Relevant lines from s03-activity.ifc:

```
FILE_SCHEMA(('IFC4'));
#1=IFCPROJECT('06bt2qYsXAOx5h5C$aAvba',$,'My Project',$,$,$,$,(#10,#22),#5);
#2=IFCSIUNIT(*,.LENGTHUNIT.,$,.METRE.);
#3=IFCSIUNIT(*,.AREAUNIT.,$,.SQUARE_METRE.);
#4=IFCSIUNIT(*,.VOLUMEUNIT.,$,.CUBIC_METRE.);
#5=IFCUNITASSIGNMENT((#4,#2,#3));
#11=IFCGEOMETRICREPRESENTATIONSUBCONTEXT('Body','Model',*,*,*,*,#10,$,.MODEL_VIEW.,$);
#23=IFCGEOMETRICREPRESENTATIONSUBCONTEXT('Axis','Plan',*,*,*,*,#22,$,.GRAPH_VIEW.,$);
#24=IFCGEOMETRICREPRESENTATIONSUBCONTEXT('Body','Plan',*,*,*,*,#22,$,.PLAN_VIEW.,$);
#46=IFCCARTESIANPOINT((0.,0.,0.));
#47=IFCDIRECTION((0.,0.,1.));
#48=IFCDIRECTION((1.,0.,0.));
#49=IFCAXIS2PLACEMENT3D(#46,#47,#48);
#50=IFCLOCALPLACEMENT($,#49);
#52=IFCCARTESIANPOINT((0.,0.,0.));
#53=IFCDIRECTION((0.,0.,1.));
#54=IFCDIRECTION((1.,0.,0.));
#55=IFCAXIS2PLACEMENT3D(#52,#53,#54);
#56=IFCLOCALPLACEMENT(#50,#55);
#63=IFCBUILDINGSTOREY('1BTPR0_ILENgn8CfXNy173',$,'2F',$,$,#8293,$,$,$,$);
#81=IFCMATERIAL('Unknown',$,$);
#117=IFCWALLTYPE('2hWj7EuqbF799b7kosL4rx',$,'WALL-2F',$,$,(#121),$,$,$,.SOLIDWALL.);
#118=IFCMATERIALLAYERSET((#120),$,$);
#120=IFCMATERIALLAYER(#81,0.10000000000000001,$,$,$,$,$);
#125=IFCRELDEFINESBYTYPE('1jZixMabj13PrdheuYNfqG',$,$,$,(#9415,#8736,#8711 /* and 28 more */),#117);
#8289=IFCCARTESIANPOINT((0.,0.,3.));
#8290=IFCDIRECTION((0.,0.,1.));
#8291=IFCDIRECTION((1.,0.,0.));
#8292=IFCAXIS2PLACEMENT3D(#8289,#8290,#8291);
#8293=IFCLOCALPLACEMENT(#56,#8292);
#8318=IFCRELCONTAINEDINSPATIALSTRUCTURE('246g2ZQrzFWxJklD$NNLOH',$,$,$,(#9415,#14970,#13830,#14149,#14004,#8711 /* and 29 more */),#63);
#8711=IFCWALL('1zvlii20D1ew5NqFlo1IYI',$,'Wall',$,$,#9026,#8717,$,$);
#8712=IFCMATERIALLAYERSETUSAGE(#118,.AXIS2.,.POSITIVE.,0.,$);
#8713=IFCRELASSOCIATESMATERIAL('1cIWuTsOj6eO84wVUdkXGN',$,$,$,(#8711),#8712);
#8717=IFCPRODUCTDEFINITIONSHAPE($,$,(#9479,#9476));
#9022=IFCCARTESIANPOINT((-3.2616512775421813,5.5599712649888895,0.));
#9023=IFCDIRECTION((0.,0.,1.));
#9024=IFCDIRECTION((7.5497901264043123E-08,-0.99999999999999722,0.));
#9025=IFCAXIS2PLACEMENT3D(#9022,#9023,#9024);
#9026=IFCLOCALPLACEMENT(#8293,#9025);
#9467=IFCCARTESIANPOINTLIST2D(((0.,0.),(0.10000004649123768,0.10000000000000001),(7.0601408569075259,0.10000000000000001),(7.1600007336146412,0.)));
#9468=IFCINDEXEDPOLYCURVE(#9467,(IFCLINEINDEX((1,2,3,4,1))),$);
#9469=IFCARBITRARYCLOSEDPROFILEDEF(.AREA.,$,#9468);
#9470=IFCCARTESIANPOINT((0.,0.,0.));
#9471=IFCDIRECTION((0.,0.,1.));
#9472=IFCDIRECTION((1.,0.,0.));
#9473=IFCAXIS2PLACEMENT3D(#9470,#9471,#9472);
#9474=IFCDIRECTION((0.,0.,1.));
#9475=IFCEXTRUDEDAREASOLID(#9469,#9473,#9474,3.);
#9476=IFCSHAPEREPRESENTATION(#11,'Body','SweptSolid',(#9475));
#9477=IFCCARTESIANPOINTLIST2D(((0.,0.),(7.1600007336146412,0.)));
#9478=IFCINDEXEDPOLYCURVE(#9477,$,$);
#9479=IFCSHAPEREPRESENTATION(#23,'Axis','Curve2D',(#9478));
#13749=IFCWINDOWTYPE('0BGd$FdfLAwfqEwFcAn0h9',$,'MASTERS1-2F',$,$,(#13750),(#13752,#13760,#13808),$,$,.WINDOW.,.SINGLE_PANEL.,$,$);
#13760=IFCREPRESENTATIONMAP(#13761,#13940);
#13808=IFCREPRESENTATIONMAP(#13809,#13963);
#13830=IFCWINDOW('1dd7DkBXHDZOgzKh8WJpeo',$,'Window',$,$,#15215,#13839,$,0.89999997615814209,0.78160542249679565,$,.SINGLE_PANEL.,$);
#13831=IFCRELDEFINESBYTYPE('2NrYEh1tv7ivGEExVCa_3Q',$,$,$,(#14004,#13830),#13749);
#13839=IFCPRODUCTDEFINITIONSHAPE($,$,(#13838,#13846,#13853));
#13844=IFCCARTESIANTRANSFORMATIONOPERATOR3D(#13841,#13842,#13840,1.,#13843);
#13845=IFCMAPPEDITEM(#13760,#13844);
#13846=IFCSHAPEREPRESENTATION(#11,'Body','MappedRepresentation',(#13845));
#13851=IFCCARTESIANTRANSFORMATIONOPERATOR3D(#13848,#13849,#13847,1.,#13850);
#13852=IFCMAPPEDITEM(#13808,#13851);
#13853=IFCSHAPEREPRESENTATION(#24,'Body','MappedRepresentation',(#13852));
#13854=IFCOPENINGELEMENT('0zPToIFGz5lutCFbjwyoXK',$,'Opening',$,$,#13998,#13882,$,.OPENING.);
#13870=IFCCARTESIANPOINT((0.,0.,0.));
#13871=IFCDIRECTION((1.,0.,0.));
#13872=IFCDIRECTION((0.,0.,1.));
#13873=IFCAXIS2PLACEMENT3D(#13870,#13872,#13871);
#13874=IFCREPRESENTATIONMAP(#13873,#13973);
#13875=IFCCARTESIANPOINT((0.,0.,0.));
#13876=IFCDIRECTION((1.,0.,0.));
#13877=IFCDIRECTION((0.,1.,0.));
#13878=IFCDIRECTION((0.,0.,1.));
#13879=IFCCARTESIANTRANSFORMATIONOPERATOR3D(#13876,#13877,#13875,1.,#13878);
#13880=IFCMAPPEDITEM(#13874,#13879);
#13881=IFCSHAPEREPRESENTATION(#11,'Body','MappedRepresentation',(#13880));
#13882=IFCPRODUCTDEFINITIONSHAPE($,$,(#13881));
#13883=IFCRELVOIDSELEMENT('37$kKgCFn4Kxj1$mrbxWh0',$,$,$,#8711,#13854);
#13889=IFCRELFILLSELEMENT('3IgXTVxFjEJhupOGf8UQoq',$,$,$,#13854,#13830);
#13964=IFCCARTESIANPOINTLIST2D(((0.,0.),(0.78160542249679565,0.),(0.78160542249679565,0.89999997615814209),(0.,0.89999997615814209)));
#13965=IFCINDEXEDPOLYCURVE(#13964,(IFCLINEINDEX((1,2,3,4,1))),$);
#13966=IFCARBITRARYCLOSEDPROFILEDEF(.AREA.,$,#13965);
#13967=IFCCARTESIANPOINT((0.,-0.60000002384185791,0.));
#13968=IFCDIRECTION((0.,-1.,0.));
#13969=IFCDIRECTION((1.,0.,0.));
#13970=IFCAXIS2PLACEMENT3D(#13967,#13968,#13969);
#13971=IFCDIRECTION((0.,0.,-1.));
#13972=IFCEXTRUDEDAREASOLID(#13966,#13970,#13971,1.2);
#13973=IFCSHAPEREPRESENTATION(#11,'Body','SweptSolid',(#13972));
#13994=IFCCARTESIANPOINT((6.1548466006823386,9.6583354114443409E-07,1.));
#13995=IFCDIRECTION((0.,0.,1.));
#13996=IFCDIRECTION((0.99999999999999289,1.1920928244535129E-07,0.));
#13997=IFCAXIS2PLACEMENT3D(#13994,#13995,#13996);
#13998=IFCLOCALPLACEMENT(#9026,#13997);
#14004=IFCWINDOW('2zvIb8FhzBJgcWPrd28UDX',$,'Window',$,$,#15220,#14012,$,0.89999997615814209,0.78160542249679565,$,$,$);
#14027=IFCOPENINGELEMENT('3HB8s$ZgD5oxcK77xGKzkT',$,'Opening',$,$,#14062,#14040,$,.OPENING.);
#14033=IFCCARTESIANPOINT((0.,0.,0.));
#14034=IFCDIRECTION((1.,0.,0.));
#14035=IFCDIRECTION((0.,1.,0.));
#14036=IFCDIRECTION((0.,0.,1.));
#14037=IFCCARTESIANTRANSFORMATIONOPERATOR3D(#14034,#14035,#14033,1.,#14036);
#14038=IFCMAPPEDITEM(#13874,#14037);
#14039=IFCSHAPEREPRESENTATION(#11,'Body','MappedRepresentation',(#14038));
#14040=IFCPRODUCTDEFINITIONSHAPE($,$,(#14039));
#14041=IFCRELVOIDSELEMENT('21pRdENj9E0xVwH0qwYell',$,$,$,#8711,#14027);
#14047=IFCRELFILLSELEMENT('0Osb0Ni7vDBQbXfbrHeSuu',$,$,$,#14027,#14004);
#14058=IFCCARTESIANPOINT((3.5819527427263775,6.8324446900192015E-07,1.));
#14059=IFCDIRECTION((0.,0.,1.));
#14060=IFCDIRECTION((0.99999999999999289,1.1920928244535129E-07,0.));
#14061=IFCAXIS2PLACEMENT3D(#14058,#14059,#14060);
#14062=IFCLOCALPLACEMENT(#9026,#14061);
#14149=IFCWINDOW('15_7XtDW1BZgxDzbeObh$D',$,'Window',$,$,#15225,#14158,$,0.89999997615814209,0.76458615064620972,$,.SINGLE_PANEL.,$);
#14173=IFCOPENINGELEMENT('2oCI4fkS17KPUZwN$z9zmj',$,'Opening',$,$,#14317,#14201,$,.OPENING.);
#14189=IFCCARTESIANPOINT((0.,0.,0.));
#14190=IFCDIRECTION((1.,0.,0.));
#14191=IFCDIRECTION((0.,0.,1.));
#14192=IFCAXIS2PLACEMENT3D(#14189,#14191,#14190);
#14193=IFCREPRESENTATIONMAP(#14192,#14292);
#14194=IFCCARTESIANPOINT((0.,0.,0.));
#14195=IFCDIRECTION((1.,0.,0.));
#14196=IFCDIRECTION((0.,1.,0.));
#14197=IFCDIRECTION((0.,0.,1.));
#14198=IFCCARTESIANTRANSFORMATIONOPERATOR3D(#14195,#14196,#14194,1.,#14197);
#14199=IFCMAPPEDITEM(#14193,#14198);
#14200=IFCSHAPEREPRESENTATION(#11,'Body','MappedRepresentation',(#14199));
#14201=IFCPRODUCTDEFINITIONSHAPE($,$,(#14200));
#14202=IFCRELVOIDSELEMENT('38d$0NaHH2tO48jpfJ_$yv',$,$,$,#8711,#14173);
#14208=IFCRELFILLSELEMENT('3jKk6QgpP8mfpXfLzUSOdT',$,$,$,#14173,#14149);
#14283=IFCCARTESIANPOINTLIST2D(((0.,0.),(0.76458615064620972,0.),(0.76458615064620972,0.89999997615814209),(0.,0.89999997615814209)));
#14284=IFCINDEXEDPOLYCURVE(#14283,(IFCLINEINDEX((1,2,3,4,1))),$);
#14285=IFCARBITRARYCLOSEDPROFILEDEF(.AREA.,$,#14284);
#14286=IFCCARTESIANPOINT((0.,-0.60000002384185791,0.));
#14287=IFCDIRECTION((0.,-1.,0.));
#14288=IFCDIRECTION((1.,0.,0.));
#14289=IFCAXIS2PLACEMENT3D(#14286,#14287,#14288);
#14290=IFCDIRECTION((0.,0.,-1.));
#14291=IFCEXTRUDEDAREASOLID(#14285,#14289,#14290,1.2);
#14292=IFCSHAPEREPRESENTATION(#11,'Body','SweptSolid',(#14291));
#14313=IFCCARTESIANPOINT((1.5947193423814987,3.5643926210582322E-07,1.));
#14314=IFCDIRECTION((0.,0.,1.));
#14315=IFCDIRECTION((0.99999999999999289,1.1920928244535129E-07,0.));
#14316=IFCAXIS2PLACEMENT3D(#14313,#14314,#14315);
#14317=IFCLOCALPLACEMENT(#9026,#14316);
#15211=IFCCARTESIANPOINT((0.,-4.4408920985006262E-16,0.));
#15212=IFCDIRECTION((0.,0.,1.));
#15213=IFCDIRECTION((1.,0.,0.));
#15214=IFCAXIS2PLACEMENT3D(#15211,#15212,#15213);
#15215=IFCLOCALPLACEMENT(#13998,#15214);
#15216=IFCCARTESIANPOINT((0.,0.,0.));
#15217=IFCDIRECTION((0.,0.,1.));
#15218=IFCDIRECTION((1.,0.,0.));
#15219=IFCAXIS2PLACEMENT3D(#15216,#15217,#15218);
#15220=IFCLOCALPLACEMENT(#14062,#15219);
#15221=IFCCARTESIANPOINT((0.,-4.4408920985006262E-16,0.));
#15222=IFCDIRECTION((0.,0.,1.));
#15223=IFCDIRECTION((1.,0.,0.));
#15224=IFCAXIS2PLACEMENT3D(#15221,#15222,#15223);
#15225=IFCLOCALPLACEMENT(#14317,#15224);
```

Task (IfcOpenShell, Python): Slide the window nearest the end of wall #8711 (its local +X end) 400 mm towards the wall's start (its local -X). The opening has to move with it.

```python
import ifcopenshell
import ifcopenshell.api.geometry
import ifcopenshell.util.placement

model = ifcopenshell.open("s03-activity.ifc")

window = model.by_guid("1dd7DkBXHDZOgzKh8WJpeo")
opening = window.FillsVoids[0].RelatingOpeningElement
wall = opening.VoidsElements[0].RelatingBuildingElement

wall_matrix = ifcopenshell.util.placement.get_local_placement(wall.ObjectPlacement)
shift = wall_matrix[:3, 0] * -0.4
before = ifcopenshell.util.placement.get_local_placement(window.ObjectPlacement)[:3, 3].copy()

# The window is placed relative to its opening, so it follows when the opening moves.
matrix = ifcopenshell.util.placement.get_local_placement(opening.ObjectPlacement)
matrix[:3, 3] += shift
ifcopenshell.api.geometry.edit_object_placement(
    model, product=opening, matrix=matrix, is_si=False, should_transform_children=True
)

after = ifcopenshell.util.placement.get_local_placement(window.ObjectPlacement)[:3, 3]
print("window moved by", (after - before).round(3) + 0.0)

model.write("s03-activity_updated.ifc")
```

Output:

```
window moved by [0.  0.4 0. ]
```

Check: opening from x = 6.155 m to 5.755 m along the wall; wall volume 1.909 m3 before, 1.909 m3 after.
